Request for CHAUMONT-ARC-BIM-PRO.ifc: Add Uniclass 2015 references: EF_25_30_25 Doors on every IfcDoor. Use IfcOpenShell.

First a look at what the model holds.

```python
import ifcopenshell

model = ifcopenshell.open("CHAUMONT-ARC-BIM-PRO.ifc")
print(model.schema)
print("classifications:", [c.Name for c in model.by_type("IfcClassification")])
for ifc_class in ("IfcDoor", "IfcRoof", "IfcStair", "IfcWall", "IfcWindow"):
    print(ifc_class, len(model.by_type(ifc_class)))
```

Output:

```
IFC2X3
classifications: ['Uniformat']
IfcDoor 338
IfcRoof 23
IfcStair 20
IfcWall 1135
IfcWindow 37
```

```python
import ifcopenshell
import ifcopenshell.api.classification

model = ifcopenshell.open("CHAUMONT-ARC-BIM-PRO.ifc")

# IFC2X3 requires Source and Edition and has no link from the project to the system.
system = model.create_entity("IfcClassification", Source="NBS", Edition="2015", Name="Uniclass 2015")

codes = {
    "IfcDoor": ("EF_25_30_25", "Doors"),
}
for ifc_class, (code, name) in codes.items():
    products = model.by_type(ifc_class)
    ifcopenshell.api.classification.add_reference(
        model, products=products, classification=system, identification=code, name=name
    )
    print(code, len(products))

model.write("CHAUMONT-ARC-BIM-PRO-out.ifc")
```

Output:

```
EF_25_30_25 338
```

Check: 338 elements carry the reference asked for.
